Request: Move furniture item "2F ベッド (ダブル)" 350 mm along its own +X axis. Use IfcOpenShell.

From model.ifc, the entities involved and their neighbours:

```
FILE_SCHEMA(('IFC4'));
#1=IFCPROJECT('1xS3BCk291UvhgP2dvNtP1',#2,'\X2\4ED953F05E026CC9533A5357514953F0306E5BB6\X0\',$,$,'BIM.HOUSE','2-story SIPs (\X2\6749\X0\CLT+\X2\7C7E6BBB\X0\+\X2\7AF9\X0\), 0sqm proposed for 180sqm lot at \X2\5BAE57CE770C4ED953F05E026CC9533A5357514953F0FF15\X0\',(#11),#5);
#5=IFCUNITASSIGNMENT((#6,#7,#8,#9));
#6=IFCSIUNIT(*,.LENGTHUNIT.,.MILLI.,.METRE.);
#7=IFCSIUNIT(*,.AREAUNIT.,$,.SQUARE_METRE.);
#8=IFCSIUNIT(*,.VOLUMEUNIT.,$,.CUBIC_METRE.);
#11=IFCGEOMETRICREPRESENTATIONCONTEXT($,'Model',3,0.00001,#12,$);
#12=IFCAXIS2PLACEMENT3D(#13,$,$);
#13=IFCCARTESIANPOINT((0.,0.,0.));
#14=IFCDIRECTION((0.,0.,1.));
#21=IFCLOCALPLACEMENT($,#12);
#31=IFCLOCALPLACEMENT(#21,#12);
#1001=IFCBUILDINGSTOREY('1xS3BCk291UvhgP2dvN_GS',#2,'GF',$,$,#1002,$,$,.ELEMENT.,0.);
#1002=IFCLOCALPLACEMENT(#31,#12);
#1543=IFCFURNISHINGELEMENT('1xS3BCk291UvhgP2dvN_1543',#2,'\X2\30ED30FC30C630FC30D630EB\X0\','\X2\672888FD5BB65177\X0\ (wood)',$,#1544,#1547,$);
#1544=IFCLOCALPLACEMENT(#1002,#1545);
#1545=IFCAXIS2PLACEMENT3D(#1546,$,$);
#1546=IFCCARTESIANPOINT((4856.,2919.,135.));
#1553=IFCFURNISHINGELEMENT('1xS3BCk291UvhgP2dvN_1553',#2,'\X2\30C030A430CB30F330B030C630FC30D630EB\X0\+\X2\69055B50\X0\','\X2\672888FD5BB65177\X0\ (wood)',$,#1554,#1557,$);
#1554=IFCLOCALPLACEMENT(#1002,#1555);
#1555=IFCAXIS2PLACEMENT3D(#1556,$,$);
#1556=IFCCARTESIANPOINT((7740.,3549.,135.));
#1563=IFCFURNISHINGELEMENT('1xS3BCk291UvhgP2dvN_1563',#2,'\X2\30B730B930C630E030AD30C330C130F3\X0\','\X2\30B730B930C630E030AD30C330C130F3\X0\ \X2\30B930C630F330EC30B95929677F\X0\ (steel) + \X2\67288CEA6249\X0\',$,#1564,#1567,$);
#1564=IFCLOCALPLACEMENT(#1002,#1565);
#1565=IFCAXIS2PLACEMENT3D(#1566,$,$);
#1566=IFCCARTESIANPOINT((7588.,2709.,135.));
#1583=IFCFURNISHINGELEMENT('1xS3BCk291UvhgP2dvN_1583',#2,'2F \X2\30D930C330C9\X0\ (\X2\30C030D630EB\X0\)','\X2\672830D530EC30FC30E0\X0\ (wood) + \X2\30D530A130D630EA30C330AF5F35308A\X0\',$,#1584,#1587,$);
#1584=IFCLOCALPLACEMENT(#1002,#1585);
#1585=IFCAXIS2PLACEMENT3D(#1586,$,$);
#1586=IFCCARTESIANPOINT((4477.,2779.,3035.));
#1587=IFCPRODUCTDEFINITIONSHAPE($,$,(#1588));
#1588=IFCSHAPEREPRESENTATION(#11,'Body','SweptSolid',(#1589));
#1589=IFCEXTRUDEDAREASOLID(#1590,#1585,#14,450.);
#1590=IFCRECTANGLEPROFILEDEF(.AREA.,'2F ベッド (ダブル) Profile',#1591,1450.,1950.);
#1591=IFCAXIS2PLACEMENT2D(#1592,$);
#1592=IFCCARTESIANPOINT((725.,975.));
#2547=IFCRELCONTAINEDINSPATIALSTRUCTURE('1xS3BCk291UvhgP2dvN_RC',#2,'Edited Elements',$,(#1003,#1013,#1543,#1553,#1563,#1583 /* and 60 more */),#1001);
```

```python
import ifcopenshell
import ifcopenshell.api.geometry
import ifcopenshell.util.placement
import ifcopenshell.util.unit

model = ifcopenshell.open("model.ifc")
unit_scale = ifcopenshell.util.unit.calculate_unit_scale(model)

item = model.by_guid("1xS3BCk291UvhgP2dvN_1583")
matrix = ifcopenshell.util.placement.get_local_placement(item.ObjectPlacement)
matrix[:3, 3] += matrix[:3, 0] * 0.35 / unit_scale
ifcopenshell.api.geometry.edit_object_placement(model, product=item, matrix=matrix, is_si=False)

print(ifcopenshell.util.placement.get_local_placement(item.ObjectPlacement).round(3) + 0.0)

model.write("model_updated.ifc")
```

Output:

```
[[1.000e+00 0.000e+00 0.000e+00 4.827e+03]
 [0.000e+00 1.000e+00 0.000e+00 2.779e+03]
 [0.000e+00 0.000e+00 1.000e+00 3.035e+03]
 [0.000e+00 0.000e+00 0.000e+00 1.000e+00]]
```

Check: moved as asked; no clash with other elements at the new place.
